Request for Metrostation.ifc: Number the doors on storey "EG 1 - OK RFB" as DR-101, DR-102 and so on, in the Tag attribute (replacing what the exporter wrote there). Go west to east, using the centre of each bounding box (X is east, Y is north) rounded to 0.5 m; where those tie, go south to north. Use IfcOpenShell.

First a look at what the model holds.

```python
import ifcopenshell
import ifcopenshell.util.element
import ifcopenshell.util.placement

model = ifcopenshell.open("Metrostation.ifc")
print(model.schema)
storey = next(s for s in model.by_type("IfcBuildingStorey") if s.Name == "EG 1 - OK RFB")
doors = [e for e in ifcopenshell.util.element.get_decomposition(storey) if e.is_a("IfcDoor")]
for e in sorted(doors, key=lambda e: e.id()):
    origin = ifcopenshell.util.placement.get_local_placement(e.ObjectPlacement)[:3, 3]
    print(e.id(), e.Tag, e.Name, origin.round(2) + 0.0, sep=" | ")
```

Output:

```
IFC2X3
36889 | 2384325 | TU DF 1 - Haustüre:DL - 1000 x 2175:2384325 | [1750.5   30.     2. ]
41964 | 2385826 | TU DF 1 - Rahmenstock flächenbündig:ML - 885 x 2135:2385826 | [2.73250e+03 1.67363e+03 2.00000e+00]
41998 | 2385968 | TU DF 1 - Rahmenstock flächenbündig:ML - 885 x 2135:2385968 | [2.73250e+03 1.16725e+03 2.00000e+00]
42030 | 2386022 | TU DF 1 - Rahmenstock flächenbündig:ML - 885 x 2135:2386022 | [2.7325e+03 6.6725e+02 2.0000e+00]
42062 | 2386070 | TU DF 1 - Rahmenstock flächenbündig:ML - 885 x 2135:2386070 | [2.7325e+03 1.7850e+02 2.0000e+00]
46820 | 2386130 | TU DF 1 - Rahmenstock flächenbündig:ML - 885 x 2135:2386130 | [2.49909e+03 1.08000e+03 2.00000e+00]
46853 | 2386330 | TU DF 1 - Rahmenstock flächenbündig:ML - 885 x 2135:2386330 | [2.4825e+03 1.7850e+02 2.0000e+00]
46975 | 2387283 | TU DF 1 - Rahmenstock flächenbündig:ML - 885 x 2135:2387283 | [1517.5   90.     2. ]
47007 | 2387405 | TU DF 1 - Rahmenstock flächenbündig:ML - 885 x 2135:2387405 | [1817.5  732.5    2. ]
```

```python
import ifcopenshell
import ifcopenshell.geom
import ifcopenshell.util.element
import ifcopenshell.util.shape

model = ifcopenshell.open("Metrostation.ifc")
settings = ifcopenshell.geom.settings()
settings.set("use-world-coords", True)


def centre(element):
    shape = ifcopenshell.geom.create_shape(settings, element)
    return ifcopenshell.util.shape.get_bbox_centroid(shape.geometry)


storey = next(s for s in model.by_type("IfcBuildingStorey") if s.Name == "EG 1 - OK RFB")
doors = [e for e in ifcopenshell.util.element.get_decomposition(storey) if e.is_a("IfcDoor")]

# Insertion points can sit at a corner or the storey origin, so sort by the geometry (in metres).
centres = {e: centre(e) for e in doors}
doors.sort(key=lambda e: (round(centres[e][0] / 0.5), centres[e][1]))

for i, e in enumerate(doors, start=1):
    number = f"DR-1{i:02d}"
    e.Tag = number
    print(e.id(), number)

model.write("Metrostation_rev.ifc")
```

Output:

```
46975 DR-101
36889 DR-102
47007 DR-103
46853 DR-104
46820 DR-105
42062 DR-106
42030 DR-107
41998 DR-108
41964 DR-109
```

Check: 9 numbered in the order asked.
